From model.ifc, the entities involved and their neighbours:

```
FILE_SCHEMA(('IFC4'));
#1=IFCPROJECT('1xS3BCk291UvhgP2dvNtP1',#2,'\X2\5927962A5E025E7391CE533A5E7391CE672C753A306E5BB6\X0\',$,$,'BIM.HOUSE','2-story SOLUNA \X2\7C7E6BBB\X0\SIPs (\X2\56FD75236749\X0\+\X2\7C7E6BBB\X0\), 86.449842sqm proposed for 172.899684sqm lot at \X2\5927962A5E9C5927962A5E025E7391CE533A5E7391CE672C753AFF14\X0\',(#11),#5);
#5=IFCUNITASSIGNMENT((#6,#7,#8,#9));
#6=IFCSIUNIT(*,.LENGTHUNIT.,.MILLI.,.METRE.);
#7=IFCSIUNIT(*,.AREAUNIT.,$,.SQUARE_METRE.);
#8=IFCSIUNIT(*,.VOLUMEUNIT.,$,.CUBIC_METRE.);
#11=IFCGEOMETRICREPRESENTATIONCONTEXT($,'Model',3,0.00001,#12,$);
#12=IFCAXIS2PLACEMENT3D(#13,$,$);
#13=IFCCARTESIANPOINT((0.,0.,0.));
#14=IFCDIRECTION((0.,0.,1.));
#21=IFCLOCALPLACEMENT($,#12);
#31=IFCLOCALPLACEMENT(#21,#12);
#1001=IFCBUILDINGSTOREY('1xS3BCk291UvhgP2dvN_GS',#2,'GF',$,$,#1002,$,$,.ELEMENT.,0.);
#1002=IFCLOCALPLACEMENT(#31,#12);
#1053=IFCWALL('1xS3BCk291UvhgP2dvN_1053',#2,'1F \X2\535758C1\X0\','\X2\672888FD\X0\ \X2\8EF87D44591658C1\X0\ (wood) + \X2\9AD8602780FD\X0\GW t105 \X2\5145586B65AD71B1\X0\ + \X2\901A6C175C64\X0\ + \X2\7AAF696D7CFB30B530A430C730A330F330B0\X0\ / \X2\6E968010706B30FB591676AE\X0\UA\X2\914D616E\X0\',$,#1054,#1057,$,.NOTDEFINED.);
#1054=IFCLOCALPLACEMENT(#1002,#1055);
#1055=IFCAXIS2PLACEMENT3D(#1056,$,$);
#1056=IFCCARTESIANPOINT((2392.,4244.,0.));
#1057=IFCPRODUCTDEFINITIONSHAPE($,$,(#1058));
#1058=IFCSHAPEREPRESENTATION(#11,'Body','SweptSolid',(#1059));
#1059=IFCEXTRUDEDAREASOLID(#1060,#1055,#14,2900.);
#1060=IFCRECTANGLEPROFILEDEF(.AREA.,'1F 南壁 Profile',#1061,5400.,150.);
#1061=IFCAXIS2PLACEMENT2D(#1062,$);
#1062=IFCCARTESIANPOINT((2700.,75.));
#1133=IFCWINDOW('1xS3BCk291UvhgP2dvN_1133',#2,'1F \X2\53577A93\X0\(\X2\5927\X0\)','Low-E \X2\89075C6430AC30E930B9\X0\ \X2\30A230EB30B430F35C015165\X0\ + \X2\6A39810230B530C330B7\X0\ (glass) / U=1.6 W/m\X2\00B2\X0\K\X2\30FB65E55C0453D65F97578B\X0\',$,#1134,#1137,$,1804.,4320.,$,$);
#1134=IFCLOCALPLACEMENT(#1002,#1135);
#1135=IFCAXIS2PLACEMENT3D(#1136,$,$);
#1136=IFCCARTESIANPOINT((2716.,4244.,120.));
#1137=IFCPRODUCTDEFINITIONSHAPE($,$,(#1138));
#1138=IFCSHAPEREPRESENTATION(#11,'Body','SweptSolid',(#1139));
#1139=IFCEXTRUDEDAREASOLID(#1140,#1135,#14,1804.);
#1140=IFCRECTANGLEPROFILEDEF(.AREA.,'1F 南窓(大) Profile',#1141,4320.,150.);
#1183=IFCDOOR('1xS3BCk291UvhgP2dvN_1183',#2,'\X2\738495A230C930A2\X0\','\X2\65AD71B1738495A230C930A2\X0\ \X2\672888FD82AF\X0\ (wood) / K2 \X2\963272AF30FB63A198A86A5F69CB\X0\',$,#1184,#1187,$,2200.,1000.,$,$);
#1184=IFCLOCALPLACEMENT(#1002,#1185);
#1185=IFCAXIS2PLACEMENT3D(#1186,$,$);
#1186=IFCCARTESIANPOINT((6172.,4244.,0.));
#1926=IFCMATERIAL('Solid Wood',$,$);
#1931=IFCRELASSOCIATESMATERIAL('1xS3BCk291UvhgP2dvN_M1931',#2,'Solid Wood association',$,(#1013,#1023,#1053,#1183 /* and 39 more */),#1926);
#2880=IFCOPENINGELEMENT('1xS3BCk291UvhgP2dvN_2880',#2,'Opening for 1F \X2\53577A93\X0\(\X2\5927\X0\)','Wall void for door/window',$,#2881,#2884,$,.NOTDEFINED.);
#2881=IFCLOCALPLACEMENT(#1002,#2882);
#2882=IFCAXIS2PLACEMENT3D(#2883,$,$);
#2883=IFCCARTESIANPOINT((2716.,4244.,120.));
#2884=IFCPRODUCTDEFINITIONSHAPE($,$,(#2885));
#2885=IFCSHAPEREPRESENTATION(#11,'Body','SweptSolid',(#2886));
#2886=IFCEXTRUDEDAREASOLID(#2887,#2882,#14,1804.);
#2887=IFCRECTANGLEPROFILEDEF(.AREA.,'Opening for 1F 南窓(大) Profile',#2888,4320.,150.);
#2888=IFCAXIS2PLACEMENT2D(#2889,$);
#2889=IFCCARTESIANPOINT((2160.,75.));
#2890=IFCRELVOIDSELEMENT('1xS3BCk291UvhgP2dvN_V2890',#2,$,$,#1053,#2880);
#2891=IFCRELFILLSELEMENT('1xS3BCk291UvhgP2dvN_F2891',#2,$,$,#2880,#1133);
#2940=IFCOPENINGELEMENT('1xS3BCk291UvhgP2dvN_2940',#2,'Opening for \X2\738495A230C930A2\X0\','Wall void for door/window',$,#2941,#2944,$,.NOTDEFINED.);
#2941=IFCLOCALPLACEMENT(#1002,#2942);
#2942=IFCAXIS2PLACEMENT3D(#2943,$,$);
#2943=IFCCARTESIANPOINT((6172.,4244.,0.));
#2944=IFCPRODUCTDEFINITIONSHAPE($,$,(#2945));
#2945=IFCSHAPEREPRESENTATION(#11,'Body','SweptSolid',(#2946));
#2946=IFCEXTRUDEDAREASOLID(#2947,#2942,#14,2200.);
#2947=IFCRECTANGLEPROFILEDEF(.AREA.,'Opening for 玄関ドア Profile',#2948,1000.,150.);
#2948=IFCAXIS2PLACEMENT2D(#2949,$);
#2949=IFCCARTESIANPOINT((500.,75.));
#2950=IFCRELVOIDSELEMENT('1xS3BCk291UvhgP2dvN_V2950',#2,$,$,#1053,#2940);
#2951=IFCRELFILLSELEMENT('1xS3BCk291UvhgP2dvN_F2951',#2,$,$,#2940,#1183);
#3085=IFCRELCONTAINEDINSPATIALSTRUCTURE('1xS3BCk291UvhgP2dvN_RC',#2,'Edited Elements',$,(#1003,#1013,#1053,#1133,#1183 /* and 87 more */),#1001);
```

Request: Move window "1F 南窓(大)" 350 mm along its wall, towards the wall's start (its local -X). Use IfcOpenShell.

```python
import ifcopenshell
import ifcopenshell.api.geometry
import ifcopenshell.util.placement
import ifcopenshell.util.unit

model = ifcopenshell.open("model.ifc")
unit_scale = ifcopenshell.util.unit.calculate_unit_scale(model)

window = model.by_guid("1xS3BCk291UvhgP2dvN_1133")
opening = window.FillsVoids[0].RelatingOpeningElement
wall = opening.VoidsElements[0].RelatingBuildingElement

wall_matrix = ifcopenshell.util.placement.get_local_placement(wall.ObjectPlacement)
shift = wall_matrix[:3, 0] * -0.35 / unit_scale
before = ifcopenshell.util.placement.get_local_placement(window.ObjectPlacement)[:3, 3].copy()

# The window is not placed relative to its opening, so move both.
for product in (opening, window):
    matrix = ifcopenshell.util.placement.get_local_placement(product.ObjectPlacement)
    matrix[:3, 3] += shift
    ifcopenshell.api.geometry.edit_object_placement(model, product=product, matrix=matrix, is_si=False)

after = ifcopenshell.util.placement.get_local_placement(window.ObjectPlacement)[:3, 3]
print("window moved by", (after - before).round(3) + 0.0)

model.write("model_edited.ifc")
```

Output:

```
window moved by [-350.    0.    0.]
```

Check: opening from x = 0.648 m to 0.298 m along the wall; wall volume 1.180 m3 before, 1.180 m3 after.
